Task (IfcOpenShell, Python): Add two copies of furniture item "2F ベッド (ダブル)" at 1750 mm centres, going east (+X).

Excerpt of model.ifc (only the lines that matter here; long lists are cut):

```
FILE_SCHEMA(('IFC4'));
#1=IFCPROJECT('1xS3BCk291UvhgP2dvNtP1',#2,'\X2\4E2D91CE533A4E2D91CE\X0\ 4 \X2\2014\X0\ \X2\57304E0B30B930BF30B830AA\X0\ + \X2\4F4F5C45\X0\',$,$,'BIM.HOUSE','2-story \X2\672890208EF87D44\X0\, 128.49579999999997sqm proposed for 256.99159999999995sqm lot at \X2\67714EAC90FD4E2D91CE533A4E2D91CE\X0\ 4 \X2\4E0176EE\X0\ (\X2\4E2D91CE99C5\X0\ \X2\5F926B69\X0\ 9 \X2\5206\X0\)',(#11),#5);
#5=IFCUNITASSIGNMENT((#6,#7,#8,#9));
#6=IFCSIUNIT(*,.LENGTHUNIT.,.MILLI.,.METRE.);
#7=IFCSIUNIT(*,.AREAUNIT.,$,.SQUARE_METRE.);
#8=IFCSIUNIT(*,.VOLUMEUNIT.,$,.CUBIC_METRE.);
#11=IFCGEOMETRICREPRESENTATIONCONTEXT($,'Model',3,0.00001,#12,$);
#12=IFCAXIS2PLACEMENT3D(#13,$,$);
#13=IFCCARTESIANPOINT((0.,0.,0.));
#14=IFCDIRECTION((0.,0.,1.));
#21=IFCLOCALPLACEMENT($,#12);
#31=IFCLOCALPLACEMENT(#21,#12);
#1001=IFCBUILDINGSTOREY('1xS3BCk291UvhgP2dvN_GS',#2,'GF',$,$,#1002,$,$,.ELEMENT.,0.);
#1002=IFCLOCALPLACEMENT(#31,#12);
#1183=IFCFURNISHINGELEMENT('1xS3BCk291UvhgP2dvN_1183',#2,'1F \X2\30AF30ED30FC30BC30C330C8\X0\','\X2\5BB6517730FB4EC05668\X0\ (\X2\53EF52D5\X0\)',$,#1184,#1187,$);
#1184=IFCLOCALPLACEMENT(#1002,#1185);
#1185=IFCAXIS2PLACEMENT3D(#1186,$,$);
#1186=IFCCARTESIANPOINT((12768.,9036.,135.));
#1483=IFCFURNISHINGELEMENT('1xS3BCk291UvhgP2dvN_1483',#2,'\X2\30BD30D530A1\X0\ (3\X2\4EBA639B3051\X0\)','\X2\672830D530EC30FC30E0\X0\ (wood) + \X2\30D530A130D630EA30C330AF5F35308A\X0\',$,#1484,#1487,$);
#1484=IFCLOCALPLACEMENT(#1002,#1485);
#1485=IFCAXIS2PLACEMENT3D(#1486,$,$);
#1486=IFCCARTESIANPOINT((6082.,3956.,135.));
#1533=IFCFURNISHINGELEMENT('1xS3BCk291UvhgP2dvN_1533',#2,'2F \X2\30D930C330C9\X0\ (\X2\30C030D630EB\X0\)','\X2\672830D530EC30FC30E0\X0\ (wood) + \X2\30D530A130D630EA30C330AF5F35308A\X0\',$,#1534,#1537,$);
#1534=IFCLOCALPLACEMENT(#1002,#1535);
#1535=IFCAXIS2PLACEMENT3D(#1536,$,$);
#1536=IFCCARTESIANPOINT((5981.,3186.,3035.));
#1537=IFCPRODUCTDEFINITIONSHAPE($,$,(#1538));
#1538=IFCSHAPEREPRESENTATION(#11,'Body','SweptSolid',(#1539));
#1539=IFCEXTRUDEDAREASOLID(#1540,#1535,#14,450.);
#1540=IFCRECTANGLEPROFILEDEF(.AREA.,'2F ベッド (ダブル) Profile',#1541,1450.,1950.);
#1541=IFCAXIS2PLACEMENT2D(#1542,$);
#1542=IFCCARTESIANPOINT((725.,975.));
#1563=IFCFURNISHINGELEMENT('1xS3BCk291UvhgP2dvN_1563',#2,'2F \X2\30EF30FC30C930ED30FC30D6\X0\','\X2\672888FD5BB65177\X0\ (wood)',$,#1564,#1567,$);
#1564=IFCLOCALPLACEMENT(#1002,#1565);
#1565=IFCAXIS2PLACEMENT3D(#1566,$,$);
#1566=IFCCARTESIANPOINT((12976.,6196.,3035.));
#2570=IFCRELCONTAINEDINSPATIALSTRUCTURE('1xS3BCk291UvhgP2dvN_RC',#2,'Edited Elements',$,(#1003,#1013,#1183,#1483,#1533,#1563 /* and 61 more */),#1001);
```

```python
import numpy as np
import ifcopenshell
import ifcopenshell.api.geometry
import ifcopenshell.api.root
import ifcopenshell.util.element
import ifcopenshell.util.placement
import ifcopenshell.util.unit

model = ifcopenshell.open("model.ifc")
unit_scale = ifcopenshell.util.unit.calculate_unit_scale(model)


def reuse_history(source, copy):
    """copy_class also copies each property set's owner history, people and application; keep the originals."""
    for rel in copy.IsDefinedBy:
        if rel.is_a("IfcRelDefinesByProperties") and (history := rel.RelatingPropertyDefinition.OwnerHistory):
            rel.RelatingPropertyDefinition.OwnerHistory = source.OwnerHistory
            ifcopenshell.util.element.remove_deep2(model, history)


source = model.by_guid("1xS3BCk291UvhgP2dvN_1533")
base = ifcopenshell.util.placement.get_local_placement(source.ObjectPlacement)
step = np.array([1.0, 0.0, 0.0]) * 1.75 / unit_scale

for i in range(1, 3):
    copy = ifcopenshell.api.root.copy_class(model, product=source)
    copy.Representation = ifcopenshell.util.element.copy_deep(
        model, source.Representation, exclude=["IfcGeometricRepresentationContext", "IfcRepresentationMap"]
    )
    reuse_history(source, copy)
    matrix = base.copy()
    matrix[:3, 3] += i * step
    print("added at", matrix[:3, 3].round(3) + 0.0)
    ifcopenshell.api.geometry.edit_object_placement(model, product=copy, matrix=matrix, is_si=False)

model.write("model_v2.ifc")
```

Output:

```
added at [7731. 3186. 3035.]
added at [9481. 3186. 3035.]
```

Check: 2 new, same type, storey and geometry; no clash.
